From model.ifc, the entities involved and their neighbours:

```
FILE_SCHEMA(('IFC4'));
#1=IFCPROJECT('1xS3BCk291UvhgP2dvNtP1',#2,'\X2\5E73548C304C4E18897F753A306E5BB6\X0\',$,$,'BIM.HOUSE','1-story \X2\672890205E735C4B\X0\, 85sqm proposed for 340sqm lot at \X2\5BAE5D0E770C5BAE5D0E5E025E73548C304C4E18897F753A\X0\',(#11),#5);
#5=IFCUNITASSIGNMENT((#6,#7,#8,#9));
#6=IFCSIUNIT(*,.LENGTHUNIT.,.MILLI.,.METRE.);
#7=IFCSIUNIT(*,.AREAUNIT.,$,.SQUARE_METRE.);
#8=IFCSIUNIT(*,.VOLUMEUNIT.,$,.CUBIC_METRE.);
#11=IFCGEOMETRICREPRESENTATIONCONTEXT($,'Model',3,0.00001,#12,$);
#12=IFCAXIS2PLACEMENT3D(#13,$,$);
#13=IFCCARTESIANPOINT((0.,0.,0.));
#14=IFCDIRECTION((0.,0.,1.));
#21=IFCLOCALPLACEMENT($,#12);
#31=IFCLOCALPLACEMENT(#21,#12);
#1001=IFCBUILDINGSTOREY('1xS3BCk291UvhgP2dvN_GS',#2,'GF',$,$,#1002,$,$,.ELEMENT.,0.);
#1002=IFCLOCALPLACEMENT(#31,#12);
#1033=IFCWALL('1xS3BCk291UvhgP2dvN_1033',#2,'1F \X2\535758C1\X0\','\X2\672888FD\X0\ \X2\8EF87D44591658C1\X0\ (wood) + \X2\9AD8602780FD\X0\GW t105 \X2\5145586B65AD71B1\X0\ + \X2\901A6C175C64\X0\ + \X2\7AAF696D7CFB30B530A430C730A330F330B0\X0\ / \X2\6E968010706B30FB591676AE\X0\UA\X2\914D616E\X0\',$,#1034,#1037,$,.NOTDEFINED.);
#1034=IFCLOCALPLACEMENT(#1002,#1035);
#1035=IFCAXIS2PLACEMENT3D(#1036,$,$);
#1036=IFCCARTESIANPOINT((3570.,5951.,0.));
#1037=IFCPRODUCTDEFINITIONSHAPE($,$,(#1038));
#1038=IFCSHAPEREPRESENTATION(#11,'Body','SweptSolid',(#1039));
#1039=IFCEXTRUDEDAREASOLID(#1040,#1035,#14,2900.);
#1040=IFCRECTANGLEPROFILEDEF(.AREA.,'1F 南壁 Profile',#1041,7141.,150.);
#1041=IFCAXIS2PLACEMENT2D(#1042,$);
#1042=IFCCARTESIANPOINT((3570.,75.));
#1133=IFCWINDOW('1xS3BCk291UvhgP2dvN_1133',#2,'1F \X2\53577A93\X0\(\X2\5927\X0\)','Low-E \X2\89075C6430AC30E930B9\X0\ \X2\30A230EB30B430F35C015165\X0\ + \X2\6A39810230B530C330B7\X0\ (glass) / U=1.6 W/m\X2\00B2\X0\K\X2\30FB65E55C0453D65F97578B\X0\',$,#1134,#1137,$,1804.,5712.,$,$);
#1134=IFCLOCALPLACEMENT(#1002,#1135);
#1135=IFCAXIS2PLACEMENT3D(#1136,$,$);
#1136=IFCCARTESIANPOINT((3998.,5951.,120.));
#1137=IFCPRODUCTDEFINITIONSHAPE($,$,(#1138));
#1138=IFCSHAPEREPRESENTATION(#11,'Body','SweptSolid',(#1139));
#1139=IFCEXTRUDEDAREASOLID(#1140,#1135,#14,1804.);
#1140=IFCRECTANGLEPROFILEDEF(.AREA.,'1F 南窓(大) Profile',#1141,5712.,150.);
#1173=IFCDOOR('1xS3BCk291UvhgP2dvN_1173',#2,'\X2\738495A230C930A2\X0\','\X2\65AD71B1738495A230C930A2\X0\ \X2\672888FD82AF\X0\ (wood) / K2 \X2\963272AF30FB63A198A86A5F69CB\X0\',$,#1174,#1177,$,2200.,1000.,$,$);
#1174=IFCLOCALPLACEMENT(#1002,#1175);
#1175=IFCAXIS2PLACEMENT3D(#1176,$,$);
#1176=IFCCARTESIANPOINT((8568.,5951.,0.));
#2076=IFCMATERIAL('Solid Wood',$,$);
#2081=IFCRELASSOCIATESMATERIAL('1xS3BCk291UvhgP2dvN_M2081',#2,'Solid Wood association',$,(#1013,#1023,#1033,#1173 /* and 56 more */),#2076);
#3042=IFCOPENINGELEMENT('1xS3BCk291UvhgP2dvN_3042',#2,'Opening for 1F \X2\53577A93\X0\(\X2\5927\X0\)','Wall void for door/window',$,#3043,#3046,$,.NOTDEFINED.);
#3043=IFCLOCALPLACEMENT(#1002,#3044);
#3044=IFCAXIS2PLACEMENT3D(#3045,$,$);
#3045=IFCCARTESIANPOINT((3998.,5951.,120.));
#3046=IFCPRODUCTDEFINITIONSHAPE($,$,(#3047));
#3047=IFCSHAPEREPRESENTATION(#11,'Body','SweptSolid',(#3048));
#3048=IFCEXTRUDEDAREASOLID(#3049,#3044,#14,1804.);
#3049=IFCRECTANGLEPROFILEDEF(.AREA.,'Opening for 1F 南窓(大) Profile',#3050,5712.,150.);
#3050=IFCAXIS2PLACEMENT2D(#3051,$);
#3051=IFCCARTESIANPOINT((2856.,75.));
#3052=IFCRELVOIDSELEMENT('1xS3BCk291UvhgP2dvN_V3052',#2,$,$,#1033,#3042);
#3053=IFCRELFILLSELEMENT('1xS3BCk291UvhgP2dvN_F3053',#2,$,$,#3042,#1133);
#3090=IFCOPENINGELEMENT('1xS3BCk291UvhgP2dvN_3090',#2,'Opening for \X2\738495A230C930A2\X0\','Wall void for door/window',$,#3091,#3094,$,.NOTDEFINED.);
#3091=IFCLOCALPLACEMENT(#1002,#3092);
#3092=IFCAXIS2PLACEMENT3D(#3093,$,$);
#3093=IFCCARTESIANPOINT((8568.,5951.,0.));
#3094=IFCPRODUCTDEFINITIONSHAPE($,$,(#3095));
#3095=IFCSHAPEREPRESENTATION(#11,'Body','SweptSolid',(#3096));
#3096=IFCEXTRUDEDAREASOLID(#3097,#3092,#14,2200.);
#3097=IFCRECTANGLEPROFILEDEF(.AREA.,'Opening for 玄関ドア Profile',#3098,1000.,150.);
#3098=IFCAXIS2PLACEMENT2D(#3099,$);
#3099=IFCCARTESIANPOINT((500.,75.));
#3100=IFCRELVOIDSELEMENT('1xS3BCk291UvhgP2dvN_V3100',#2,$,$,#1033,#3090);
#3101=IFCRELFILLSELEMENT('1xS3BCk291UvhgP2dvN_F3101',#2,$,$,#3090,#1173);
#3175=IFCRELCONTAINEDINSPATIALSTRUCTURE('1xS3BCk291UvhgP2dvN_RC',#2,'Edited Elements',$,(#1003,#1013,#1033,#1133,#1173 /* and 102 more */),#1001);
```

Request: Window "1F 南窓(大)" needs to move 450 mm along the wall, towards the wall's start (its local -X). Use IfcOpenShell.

```python
import ifcopenshell
import ifcopenshell.api.geometry
import ifcopenshell.util.placement
import ifcopenshell.util.unit

model = ifcopenshell.open("model.ifc")
unit_scale = ifcopenshell.util.unit.calculate_unit_scale(model)

window = model.by_guid("1xS3BCk291UvhgP2dvN_1133")
opening = window.FillsVoids[0].RelatingOpeningElement
wall = opening.VoidsElements[0].RelatingBuildingElement

wall_matrix = ifcopenshell.util.placement.get_local_placement(wall.ObjectPlacement)
shift = wall_matrix[:3, 0] * -0.45 / unit_scale
before = ifcopenshell.util.placement.get_local_placement(window.ObjectPlacement)[:3, 3].copy()

# The window is not placed relative to its opening, so move both.
for product in (opening, window):
    matrix = ifcopenshell.util.placement.get_local_placement(product.ObjectPlacement)
    matrix[:3, 3] += shift
    ifcopenshell.api.geometry.edit_object_placement(model, product=product, matrix=matrix, is_si=False)

after = ifcopenshell.util.placement.get_local_placement(window.ObjectPlacement)[:3, 3]
print("window moved by", (after - before).round(3) + 0.0)

model.write("model-out.ifc")
```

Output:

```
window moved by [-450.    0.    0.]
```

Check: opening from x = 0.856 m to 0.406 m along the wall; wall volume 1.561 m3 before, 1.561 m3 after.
